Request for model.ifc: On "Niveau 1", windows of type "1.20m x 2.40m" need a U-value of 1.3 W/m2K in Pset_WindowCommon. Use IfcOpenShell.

First a look at what the model holds.

```python
import ifcopenshell
import ifcopenshell.util.element

model = ifcopenshell.open("model.ifc")
print(model.schema)
storey = next(s for s in model.by_type("IfcBuildingStorey") if s.Name == "Niveau 1")
windows = [e for e in ifcopenshell.util.element.get_decomposition(storey) if e.is_a("IfcWindow")]
seen = {}
for e in windows:
    element_type = ifcopenshell.util.element.get_type(e)
    key = (element_type.Name if element_type != e and element_type else None, ifcopenshell.util.element.get_pset(e, "Pset_WindowCommon", "ThermalTransmittance"))
    seen[key] = seen.get(key, 0) + 1
for (name, value), count in sorted(seen.items(), key=str):
    print(count, "x", name, "|", value)
```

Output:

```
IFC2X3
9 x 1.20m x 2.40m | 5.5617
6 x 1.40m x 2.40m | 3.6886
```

```python
import ifcopenshell
import ifcopenshell.api.pset
import ifcopenshell.util.element

model = ifcopenshell.open("model.ifc")

storey = next(s for s in model.by_type("IfcBuildingStorey") if s.Name == "Niveau 1")
windows = [e for e in ifcopenshell.util.element.get_decomposition(storey) if e.is_a("IfcWindow")]

count = 0
for e in windows:
    element_type = ifcopenshell.util.element.get_type(e)
    if element_type in (None, e) or element_type.Name != "1.20m x 2.40m":
        continue
    # add_pset returns the element's existing set when there is one.
    pset = ifcopenshell.api.pset.add_pset(model, product=e, name="Pset_WindowCommon")
    ifcopenshell.api.pset.edit_pset(model, pset=pset, properties={"ThermalTransmittance": 1.3})
    count += 1

print(count, "windows updated")

model.write("model_rev.ifc")
```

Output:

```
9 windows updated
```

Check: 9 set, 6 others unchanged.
